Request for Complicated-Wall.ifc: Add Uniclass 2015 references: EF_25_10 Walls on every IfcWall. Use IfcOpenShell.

First a look at what the model holds.

```python
import ifcopenshell

model = ifcopenshell.open("Complicated-Wall.ifc")
print(model.schema)
print("classifications:", [c.Name for c in model.by_type("IfcClassification")])
for ifc_class in ("IfcDoor", "IfcRoof", "IfcStair", "IfcWall", "IfcWindow"):
    print(ifc_class, len(model.by_type(ifc_class)))
```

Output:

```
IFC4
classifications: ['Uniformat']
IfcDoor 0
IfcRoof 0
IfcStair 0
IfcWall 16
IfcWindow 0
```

```python
import ifcopenshell
import ifcopenshell.api.classification

model = ifcopenshell.open("Complicated-Wall.ifc")

system = ifcopenshell.api.classification.add_classification(model, classification="Uniclass 2015")

codes = {
    "IfcWall": ("EF_25_10", "Walls"),
}
for ifc_class, (code, name) in codes.items():
    products = model.by_type(ifc_class)
    ifcopenshell.api.classification.add_reference(
        model, products=products, classification=system, identification=code, name=name
    )
    print(code, len(products))

model.write("Complicated-Wall_updated.ifc")
```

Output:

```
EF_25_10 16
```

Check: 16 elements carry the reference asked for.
